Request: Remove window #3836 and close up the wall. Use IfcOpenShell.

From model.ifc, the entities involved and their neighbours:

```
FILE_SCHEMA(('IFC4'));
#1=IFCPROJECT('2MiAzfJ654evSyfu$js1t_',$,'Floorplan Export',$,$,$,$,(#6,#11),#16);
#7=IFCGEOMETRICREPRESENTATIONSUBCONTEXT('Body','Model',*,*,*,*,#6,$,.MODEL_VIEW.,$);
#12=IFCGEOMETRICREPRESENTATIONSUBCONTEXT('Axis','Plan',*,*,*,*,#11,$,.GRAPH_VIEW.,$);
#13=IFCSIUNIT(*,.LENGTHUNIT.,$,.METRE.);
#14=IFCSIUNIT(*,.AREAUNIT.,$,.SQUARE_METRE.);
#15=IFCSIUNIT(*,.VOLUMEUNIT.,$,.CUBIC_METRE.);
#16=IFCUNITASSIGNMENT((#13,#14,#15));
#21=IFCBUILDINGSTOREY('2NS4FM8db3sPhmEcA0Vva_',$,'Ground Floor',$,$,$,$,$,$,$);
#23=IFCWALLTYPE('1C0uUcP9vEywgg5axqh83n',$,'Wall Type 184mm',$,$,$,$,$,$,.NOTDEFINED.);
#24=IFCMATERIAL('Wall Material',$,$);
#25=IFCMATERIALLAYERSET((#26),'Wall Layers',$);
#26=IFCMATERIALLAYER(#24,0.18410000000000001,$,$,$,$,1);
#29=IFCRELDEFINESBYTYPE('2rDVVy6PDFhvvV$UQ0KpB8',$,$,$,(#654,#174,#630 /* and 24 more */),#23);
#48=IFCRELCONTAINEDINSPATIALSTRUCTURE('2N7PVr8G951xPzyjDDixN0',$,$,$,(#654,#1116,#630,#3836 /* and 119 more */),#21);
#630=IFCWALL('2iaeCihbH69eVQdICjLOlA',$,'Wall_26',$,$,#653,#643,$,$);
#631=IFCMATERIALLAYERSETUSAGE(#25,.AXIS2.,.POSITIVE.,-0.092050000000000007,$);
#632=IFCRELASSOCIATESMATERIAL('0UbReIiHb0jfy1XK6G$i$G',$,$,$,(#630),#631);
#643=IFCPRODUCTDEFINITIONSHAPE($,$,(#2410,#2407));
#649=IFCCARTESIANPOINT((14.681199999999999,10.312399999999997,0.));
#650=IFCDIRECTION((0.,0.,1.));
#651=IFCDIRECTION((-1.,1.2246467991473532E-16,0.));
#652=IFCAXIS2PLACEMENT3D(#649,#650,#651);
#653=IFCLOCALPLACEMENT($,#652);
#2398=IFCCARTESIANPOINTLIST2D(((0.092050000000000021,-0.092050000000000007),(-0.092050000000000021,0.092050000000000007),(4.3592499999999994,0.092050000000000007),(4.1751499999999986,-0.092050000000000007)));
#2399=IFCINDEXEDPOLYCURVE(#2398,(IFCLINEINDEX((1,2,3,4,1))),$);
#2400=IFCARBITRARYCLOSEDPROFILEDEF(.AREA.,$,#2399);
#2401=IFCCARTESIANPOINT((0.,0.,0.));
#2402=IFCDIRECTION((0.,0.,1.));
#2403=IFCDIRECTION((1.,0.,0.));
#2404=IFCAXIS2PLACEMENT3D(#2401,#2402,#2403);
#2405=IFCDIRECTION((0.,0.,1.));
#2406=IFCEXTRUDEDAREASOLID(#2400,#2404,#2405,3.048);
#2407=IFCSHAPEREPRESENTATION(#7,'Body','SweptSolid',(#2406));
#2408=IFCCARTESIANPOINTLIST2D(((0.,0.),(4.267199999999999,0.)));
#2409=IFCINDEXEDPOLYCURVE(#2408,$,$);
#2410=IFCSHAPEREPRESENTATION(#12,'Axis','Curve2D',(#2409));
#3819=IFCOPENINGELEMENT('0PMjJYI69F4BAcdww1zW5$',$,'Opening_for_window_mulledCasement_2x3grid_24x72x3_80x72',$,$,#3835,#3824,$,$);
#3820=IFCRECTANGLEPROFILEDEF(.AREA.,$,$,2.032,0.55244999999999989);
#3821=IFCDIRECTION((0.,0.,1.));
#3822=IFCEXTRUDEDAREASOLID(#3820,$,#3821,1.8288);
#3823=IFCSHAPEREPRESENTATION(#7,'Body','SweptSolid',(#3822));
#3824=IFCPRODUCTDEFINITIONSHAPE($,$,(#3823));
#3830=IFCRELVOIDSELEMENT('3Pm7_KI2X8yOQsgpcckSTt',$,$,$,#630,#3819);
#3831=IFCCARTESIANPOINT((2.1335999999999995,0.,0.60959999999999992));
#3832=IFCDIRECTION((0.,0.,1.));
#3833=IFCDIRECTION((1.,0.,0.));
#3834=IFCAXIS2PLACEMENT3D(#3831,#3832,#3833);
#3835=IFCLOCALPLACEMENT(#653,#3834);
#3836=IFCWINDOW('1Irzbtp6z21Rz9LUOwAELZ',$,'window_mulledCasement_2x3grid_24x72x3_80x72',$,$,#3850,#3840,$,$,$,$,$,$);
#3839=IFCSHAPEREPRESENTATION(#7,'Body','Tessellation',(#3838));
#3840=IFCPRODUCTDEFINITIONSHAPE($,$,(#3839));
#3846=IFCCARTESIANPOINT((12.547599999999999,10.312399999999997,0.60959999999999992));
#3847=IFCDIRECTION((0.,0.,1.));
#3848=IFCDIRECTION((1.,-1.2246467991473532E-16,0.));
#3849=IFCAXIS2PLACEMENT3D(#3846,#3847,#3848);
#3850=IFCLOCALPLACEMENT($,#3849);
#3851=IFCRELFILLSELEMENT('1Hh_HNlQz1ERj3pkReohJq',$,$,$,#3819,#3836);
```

```python
import ifcopenshell
import ifcopenshell.api.feature
import ifcopenshell.api.root
import ifcopenshell.geom
import ifcopenshell.util.shape

model = ifcopenshell.open("model.ifc")
settings = ifcopenshell.geom.settings()


def volume(element):
    """Net volume in cubic metres, openings subtracted."""
    shape = ifcopenshell.geom.create_shape(settings, element)
    return ifcopenshell.util.shape.get_volume(shape.geometry)


window = model.by_guid("1Irzbtp6z21Rz9LUOwAELZ")
opening = window.FillsVoids[0].RelatingOpeningElement
wall = opening.VoidsElements[0].RelatingBuildingElement
before = volume(wall)

ifcopenshell.api.root.remove_product(model, product=window)
ifcopenshell.api.feature.remove_feature(model, feature=opening)

after = volume(wall)

print(f"wall volume {before:.3f} -> {after:.3f} m3")

model.write("model_v2.ifc")
```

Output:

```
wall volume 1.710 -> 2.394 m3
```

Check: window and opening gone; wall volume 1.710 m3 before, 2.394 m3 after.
